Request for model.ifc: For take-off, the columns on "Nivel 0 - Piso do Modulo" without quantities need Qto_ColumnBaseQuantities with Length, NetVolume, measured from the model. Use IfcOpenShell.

First a look at what the model holds.

```python
import ifcopenshell
import ifcopenshell.util.element
import ifcopenshell.util.unit

model = ifcopenshell.open("model.ifc")
print(model.schema)
for unit_type in ("LENGTHUNIT", "AREAUNIT", "VOLUMEUNIT"):
    print(unit_type, ifcopenshell.util.unit.calculate_unit_scale(model, unit_type))
storey = next(s for s in model.by_type("IfcBuildingStorey") if s.Name == "Nivel 0 - Piso do Modulo")
columns = [e for e in ifcopenshell.util.element.get_decomposition(storey) if e.is_a("IfcColumn")]
for e in sorted(columns, key=lambda e: e.id()):
    print(e.id(), e.is_a(), e.Name, list(ifcopenshell.util.element.get_psets(e, qtos_only=True)), sep=" | ")
```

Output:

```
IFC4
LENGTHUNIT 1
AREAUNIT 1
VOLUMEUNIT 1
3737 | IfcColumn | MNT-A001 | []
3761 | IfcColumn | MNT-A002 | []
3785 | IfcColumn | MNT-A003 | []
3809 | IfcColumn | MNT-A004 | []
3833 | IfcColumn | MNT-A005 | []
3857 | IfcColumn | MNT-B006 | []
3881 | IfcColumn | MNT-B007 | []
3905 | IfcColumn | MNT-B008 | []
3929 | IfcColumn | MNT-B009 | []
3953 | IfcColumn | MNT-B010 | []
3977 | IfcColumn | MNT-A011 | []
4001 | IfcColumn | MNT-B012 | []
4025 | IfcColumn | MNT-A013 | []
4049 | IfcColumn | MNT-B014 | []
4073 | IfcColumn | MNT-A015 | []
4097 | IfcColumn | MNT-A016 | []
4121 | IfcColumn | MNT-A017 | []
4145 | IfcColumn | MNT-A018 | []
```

```python
import ifcopenshell
import ifcopenshell.api.pset
import ifcopenshell.geom
import ifcopenshell.util.element
import ifcopenshell.util.shape
import ifcopenshell.util.unit

model = ifcopenshell.open("model.ifc")
unit_scale = ifcopenshell.util.unit.calculate_unit_scale(model)
volume_scale = ifcopenshell.util.unit.calculate_unit_scale(model, "VOLUMEUNIT")
settings = ifcopenshell.geom.settings()

storey = next(s for s in model.by_type("IfcBuildingStorey") if s.Name == "Nivel 0 - Piso do Modulo")
columns = [e for e in ifcopenshell.util.element.get_decomposition(storey) if e.is_a("IfcColumn")]

for e in sorted(columns, key=lambda e: e.id()):
    if ifcopenshell.util.element.get_psets(e, qtos_only=True, should_inherit=False):
        continue
    # Geometry comes back in metres, in the element's own axes.
    shape = ifcopenshell.geom.create_shape(settings, e)
    values = {
        "Length": ifcopenshell.util.shape.get_z(shape.geometry) / unit_scale,
        "NetVolume": ifcopenshell.util.shape.get_volume(shape.geometry) / volume_scale,
    }
    qto = ifcopenshell.api.pset.add_qto(model, product=e, name="Qto_ColumnBaseQuantities")
    ifcopenshell.api.pset.edit_qto(model, qto=qto, properties=values)
    print(e.id(), {k: round(v, 3) for k, v in values.items()})

model.write("model_edited.ifc")
```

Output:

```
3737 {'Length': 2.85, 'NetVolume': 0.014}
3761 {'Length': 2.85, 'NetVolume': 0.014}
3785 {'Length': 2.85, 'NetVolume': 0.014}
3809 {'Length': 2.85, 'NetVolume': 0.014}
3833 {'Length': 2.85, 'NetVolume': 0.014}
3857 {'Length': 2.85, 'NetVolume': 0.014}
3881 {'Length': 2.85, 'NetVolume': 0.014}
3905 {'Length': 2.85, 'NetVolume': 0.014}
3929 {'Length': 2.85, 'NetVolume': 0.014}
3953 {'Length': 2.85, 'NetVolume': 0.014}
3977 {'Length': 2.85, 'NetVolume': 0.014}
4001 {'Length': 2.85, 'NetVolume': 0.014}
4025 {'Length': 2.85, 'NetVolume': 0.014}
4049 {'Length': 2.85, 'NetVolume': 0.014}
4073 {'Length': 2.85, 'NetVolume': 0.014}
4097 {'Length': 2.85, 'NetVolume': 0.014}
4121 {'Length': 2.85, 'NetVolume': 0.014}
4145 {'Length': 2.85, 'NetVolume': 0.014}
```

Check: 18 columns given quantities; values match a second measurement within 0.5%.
